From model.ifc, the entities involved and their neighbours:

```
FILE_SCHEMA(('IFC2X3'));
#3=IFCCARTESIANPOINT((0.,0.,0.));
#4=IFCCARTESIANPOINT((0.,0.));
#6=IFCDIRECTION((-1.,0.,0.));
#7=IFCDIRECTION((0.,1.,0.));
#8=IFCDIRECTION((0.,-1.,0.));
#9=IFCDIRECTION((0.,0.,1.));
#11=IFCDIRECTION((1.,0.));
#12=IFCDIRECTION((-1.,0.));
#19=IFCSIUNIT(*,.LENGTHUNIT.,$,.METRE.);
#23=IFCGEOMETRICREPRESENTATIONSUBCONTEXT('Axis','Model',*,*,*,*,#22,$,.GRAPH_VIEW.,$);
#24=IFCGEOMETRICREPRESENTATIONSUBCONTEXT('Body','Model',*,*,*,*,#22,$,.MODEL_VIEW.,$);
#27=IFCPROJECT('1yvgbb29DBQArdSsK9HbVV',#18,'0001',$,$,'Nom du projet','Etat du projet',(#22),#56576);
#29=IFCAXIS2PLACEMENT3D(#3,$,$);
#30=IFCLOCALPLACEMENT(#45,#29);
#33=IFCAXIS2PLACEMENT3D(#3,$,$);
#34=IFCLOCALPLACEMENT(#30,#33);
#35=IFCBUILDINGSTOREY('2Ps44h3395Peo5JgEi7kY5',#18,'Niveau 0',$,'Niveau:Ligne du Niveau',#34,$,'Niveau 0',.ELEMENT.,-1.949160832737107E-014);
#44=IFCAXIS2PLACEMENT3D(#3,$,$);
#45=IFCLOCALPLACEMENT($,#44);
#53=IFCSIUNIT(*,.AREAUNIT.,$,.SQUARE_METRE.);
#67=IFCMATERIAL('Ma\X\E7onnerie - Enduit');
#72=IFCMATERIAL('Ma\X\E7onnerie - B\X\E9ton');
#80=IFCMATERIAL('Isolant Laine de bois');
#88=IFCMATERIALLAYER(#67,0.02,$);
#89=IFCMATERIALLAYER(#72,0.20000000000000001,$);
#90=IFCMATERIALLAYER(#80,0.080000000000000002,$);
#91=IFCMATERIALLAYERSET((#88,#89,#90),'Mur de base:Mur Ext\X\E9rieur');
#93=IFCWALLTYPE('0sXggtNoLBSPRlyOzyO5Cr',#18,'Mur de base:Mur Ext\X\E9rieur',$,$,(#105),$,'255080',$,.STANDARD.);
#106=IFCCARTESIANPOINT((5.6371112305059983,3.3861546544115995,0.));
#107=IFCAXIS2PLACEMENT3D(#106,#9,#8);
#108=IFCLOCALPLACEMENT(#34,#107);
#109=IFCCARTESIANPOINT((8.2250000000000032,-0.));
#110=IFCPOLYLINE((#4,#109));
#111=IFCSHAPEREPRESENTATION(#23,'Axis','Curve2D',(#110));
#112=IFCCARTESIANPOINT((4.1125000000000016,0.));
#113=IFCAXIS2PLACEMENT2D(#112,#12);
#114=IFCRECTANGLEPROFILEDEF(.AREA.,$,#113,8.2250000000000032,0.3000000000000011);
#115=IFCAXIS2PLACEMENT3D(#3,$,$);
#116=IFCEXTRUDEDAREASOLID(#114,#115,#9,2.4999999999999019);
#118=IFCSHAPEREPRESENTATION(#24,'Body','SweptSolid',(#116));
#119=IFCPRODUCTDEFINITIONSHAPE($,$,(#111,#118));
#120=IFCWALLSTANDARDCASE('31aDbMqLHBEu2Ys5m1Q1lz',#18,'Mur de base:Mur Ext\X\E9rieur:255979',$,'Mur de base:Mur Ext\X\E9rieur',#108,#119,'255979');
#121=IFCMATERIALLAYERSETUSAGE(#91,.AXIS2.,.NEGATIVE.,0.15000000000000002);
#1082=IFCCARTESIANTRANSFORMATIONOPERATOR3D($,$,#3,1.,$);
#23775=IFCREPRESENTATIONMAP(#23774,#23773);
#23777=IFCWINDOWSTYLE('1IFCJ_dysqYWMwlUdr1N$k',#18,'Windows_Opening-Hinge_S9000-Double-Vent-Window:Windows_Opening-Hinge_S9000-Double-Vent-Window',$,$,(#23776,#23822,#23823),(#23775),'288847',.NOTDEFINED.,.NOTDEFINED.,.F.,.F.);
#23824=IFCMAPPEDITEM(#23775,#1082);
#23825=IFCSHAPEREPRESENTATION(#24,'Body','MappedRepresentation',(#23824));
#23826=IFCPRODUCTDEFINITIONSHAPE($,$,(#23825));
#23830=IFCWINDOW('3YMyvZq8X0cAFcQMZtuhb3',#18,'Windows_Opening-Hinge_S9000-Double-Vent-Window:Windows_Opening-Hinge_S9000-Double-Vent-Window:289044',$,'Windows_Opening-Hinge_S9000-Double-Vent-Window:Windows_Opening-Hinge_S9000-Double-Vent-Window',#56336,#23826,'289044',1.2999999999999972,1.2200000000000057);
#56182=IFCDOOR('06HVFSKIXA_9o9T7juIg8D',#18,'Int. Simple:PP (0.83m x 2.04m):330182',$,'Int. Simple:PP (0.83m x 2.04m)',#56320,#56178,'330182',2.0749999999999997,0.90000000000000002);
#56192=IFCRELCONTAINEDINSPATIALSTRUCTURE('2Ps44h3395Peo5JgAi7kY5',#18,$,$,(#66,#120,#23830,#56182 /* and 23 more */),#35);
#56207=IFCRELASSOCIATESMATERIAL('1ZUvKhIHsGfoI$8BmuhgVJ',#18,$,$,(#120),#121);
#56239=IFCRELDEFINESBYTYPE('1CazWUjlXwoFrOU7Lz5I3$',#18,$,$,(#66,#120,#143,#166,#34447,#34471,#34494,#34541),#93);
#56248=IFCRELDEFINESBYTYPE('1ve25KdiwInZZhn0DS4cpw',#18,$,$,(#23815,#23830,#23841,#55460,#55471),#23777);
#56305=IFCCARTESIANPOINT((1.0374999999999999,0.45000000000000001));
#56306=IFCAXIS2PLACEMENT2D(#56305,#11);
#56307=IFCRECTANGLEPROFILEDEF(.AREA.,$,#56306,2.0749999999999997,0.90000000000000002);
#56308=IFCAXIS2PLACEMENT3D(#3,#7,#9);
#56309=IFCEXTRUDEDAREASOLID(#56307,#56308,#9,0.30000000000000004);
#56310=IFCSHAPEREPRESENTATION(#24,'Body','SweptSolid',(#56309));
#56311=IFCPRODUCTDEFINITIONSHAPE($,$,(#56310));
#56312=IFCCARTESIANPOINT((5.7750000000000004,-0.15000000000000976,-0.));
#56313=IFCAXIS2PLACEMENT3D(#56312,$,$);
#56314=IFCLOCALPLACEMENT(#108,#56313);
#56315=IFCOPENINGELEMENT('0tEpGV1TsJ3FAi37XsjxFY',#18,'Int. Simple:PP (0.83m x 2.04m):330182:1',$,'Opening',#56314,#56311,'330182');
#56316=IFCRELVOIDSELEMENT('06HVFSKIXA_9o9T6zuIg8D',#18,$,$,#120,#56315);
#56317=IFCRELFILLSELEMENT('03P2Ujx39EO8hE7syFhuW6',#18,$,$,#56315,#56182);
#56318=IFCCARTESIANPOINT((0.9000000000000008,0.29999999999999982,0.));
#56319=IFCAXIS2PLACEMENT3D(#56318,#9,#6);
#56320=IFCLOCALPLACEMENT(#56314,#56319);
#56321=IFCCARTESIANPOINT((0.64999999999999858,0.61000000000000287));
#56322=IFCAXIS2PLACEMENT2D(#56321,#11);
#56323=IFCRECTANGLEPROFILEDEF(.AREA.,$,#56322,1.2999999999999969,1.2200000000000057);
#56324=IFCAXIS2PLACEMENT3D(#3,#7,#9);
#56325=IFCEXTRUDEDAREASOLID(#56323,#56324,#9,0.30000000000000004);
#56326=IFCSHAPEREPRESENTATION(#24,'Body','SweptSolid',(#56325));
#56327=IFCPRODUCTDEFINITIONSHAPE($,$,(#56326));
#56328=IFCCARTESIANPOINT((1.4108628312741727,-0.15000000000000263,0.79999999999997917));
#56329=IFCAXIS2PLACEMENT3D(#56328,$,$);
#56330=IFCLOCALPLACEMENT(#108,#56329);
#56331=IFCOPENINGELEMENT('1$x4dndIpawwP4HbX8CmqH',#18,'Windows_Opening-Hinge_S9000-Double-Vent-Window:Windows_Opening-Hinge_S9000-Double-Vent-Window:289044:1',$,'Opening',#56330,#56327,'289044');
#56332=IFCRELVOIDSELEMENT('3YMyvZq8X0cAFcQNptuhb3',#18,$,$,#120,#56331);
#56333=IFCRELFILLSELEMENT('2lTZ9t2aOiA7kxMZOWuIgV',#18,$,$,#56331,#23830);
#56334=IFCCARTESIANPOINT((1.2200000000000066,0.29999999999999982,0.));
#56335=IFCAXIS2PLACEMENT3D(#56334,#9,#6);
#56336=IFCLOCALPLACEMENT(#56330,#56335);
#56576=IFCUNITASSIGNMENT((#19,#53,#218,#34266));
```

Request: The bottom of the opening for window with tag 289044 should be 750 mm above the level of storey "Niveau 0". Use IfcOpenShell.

```python
import numpy as np
import ifcopenshell
import ifcopenshell.api.geometry
import ifcopenshell.geom
import ifcopenshell.util.element
import ifcopenshell.util.placement
import ifcopenshell.util.shape
import ifcopenshell.util.unit

model = ifcopenshell.open("model.ifc")
unit_scale = ifcopenshell.util.unit.calculate_unit_scale(model)

window = model.by_id(23830)
opening = window.FillsVoids[0].RelatingOpeningElement
storey = ifcopenshell.util.element.get_container(window, ifc_class="IfcBuildingStorey")
level = ifcopenshell.util.placement.get_local_placement(storey.ObjectPlacement)[2, 3]

# The opening's origin need not be at the sill, so measure its lowest point.
shape = ifcopenshell.geom.create_shape(ifcopenshell.geom.settings(), opening)
bottom = ifcopenshell.util.shape.get_shape_bottom_elevation(shape, shape.geometry) / unit_scale
dz = level + 0.75 / unit_scale - bottom

shift = np.array([0.0, 0.0, dz])
# The window is placed relative to its opening, so it follows when the opening moves.
matrix = ifcopenshell.util.placement.get_local_placement(opening.ObjectPlacement)
matrix[:3, 3] += shift
ifcopenshell.api.geometry.edit_object_placement(
    model, product=opening, matrix=matrix, is_si=False, should_transform_children=True
)

print(f"moved by {dz * unit_scale:+.3f} m")

model.write("model_rev.ifc")
```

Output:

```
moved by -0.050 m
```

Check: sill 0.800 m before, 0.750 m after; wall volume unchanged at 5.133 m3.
